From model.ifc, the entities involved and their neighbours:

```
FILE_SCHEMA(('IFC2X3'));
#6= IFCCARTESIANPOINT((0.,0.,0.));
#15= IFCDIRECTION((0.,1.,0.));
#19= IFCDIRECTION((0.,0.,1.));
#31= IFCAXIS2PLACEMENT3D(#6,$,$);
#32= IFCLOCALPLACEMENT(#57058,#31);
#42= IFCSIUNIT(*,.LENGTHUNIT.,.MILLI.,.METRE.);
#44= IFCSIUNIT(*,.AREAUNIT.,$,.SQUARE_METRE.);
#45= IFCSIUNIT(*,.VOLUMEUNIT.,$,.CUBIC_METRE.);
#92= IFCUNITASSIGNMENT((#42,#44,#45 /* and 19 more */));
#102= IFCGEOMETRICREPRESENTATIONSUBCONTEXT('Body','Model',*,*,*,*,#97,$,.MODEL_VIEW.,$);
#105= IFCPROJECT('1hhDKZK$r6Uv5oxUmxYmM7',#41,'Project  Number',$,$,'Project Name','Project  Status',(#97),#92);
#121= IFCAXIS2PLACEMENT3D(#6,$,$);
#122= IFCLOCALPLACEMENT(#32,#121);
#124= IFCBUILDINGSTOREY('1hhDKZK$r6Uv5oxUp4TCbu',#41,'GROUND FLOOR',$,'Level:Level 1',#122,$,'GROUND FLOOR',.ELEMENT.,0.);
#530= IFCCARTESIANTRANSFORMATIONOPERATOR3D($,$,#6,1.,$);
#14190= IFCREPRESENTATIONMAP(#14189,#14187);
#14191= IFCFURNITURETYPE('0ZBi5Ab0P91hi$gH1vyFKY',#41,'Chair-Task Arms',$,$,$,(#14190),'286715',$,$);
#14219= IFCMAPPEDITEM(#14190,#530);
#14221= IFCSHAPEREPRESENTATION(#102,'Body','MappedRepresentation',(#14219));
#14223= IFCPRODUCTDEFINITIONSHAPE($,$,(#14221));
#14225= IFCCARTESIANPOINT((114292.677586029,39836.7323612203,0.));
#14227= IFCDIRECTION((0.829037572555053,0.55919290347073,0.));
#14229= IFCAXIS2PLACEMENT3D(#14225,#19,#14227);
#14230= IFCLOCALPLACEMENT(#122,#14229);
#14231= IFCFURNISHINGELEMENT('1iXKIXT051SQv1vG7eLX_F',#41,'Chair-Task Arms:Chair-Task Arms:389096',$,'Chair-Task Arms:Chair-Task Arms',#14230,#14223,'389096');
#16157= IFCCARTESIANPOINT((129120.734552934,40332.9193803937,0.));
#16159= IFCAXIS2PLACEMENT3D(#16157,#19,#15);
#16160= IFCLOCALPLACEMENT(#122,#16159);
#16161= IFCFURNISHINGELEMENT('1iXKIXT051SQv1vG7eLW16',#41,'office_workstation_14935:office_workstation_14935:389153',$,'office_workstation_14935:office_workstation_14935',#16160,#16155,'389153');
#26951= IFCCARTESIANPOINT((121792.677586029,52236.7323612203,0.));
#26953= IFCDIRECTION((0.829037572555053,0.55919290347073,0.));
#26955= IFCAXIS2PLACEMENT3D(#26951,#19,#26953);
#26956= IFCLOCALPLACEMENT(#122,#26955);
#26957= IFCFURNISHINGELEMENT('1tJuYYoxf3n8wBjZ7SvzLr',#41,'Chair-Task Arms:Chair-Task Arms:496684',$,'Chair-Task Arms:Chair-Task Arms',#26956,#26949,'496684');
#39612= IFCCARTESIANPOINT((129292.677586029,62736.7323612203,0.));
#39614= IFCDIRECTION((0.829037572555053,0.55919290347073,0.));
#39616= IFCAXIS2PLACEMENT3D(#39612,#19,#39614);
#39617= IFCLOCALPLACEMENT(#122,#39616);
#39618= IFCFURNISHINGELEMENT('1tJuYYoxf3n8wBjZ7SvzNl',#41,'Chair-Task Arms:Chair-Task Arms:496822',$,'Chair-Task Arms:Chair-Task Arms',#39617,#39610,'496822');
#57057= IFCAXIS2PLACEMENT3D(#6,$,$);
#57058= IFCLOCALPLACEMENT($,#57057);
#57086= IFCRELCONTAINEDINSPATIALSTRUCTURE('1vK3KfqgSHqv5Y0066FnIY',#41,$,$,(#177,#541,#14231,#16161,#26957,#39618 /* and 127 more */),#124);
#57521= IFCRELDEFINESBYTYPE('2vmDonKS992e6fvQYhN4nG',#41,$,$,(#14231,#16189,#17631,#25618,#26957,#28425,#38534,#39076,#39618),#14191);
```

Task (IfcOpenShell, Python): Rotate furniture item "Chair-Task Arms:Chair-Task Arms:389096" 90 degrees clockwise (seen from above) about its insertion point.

```python
import ifcopenshell
import ifcopenshell.api.geometry
import ifcopenshell.util.placement

model = ifcopenshell.open("model.ifc")

item = model.by_id(14231)
matrix = ifcopenshell.util.placement.get_local_placement(item.ObjectPlacement)
matrix = matrix @ ifcopenshell.util.placement.rotation(-90, "Z")
ifcopenshell.api.geometry.edit_object_placement(model, product=item, matrix=matrix, is_si=False)

print(ifcopenshell.util.placement.get_local_placement(item.ObjectPlacement).round(3) + 0.0)

model.write("model_v2.ifc")
```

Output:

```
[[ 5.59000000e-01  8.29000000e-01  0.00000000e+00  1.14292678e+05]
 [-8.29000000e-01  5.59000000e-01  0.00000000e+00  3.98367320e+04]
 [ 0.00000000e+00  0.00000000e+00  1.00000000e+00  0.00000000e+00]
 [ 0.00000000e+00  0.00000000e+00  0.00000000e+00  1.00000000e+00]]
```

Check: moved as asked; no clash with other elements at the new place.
